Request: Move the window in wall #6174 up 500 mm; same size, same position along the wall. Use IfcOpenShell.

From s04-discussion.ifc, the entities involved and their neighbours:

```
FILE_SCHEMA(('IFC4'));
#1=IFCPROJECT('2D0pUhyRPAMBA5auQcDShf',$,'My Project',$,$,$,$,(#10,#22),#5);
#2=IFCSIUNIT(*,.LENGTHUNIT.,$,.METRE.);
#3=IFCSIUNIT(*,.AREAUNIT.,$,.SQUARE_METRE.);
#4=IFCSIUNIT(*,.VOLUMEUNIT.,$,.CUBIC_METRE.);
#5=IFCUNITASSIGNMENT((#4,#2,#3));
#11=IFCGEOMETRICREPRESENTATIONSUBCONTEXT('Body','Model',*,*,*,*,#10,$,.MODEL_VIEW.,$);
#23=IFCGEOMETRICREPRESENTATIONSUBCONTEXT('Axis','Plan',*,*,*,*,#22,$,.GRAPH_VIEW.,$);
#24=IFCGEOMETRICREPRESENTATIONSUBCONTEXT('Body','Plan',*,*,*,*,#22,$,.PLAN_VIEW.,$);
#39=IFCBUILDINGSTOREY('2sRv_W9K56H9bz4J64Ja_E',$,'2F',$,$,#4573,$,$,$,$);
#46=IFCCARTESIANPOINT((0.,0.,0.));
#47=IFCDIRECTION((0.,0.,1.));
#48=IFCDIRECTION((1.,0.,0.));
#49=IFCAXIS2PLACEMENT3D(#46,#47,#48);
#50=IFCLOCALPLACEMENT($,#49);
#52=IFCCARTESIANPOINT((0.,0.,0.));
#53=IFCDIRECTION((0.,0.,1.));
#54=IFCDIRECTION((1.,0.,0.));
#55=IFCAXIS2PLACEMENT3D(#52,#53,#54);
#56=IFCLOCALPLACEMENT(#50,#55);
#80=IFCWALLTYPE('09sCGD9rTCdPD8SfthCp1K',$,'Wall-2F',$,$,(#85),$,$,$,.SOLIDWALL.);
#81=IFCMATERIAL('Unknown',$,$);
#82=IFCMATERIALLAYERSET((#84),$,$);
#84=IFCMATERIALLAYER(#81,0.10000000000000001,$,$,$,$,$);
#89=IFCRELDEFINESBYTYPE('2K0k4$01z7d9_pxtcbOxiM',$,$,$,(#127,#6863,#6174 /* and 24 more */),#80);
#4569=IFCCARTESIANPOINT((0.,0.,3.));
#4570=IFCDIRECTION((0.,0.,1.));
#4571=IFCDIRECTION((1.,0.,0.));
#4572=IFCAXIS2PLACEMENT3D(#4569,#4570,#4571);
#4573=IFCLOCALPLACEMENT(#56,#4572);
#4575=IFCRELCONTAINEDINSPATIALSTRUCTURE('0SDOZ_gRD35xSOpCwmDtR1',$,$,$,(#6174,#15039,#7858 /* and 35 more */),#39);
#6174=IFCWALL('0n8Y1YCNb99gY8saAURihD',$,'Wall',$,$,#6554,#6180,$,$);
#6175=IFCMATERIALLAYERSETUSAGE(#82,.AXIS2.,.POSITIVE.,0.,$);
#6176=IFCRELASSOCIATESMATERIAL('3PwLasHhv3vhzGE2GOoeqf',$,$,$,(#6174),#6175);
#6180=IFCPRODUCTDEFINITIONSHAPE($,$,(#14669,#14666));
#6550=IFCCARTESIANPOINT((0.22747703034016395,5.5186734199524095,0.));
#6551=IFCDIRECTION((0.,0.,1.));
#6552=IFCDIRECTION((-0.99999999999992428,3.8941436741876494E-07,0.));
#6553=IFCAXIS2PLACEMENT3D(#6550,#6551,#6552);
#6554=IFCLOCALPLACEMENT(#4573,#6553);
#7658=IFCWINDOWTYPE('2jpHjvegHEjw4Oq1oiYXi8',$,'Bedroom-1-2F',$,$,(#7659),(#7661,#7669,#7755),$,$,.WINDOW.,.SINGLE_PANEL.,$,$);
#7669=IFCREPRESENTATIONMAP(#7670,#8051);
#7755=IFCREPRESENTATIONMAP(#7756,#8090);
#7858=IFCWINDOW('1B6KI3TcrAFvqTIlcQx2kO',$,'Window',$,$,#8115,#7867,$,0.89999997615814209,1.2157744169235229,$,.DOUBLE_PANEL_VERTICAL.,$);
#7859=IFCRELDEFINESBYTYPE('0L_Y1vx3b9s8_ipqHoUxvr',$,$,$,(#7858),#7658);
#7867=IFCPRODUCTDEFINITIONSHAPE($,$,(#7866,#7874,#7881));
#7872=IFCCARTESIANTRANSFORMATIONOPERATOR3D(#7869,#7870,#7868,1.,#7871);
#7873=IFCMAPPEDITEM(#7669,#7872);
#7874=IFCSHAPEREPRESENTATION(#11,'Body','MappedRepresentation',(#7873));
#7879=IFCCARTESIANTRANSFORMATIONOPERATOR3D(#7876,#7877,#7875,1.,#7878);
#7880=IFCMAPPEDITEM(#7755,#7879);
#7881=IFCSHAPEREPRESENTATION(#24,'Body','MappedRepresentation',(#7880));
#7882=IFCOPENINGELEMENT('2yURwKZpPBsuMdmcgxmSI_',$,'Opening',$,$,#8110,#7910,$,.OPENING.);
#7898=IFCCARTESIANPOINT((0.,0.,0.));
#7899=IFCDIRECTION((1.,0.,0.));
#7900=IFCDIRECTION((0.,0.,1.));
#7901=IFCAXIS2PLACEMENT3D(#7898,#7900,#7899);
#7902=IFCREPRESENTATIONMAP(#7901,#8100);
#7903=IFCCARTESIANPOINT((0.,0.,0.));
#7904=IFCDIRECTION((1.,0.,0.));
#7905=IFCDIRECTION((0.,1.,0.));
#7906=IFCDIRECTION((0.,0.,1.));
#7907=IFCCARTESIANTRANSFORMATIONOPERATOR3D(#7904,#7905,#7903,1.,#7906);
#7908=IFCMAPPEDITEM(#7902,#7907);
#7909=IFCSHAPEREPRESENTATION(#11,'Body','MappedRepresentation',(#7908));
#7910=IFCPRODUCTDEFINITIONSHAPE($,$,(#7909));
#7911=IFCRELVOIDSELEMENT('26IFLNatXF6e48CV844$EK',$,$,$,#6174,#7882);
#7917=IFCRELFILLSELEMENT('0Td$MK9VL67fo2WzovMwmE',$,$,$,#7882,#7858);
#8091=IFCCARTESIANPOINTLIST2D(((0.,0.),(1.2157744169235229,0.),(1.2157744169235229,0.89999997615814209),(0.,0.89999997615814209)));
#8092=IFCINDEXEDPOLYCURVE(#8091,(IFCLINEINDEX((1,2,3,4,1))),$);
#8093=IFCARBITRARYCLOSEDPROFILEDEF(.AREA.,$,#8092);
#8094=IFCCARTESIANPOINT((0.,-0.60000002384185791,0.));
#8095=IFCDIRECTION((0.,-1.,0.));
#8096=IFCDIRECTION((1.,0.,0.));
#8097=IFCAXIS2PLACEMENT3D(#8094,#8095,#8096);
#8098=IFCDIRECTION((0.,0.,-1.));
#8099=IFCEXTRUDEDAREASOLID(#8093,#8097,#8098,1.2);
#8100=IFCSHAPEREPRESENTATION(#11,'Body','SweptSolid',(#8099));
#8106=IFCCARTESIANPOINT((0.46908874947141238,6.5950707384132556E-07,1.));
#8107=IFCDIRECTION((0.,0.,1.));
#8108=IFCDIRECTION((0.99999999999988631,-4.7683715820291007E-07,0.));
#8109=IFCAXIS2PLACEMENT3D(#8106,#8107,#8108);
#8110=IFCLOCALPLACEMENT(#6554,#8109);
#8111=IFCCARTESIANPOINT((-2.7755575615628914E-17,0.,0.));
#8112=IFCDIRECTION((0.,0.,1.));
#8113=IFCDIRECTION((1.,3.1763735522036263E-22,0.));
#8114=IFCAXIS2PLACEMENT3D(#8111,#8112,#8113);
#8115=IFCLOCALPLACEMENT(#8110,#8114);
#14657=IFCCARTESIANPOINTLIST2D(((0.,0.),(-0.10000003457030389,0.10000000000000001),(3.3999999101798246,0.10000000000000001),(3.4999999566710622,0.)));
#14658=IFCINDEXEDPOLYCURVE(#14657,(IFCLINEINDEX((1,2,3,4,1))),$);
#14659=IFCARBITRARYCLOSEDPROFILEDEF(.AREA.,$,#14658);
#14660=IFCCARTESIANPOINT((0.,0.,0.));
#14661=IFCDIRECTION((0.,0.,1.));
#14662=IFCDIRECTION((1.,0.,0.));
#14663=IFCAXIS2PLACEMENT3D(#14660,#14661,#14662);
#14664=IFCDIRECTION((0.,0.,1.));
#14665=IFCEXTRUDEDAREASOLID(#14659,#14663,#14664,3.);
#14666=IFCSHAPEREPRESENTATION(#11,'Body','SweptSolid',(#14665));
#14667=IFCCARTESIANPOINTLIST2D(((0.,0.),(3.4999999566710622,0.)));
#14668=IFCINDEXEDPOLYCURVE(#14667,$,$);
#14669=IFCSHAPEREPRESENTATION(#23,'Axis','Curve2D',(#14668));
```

```python
import numpy as np
import ifcopenshell
import ifcopenshell.api.geometry
import ifcopenshell.util.placement
import ifcopenshell.util.unit

model = ifcopenshell.open("s04-discussion.ifc")
unit_scale = ifcopenshell.util.unit.calculate_unit_scale(model)

window = model.by_guid("1B6KI3TcrAFvqTIlcQx2kO")
opening = window.FillsVoids[0].RelatingOpeningElement
dz = 0.5

shift = np.array([0.0, 0.0, dz])
# The window is placed relative to its opening, so it follows when the opening moves.
matrix = ifcopenshell.util.placement.get_local_placement(opening.ObjectPlacement)
matrix[:3, 3] += shift
ifcopenshell.api.geometry.edit_object_placement(
    model, product=opening, matrix=matrix, is_si=False, should_transform_children=True
)

print(f"moved by {dz * unit_scale:+.3f} m")

model.write("s04-discussion_edited.ifc")
```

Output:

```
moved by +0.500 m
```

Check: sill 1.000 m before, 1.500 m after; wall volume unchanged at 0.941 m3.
